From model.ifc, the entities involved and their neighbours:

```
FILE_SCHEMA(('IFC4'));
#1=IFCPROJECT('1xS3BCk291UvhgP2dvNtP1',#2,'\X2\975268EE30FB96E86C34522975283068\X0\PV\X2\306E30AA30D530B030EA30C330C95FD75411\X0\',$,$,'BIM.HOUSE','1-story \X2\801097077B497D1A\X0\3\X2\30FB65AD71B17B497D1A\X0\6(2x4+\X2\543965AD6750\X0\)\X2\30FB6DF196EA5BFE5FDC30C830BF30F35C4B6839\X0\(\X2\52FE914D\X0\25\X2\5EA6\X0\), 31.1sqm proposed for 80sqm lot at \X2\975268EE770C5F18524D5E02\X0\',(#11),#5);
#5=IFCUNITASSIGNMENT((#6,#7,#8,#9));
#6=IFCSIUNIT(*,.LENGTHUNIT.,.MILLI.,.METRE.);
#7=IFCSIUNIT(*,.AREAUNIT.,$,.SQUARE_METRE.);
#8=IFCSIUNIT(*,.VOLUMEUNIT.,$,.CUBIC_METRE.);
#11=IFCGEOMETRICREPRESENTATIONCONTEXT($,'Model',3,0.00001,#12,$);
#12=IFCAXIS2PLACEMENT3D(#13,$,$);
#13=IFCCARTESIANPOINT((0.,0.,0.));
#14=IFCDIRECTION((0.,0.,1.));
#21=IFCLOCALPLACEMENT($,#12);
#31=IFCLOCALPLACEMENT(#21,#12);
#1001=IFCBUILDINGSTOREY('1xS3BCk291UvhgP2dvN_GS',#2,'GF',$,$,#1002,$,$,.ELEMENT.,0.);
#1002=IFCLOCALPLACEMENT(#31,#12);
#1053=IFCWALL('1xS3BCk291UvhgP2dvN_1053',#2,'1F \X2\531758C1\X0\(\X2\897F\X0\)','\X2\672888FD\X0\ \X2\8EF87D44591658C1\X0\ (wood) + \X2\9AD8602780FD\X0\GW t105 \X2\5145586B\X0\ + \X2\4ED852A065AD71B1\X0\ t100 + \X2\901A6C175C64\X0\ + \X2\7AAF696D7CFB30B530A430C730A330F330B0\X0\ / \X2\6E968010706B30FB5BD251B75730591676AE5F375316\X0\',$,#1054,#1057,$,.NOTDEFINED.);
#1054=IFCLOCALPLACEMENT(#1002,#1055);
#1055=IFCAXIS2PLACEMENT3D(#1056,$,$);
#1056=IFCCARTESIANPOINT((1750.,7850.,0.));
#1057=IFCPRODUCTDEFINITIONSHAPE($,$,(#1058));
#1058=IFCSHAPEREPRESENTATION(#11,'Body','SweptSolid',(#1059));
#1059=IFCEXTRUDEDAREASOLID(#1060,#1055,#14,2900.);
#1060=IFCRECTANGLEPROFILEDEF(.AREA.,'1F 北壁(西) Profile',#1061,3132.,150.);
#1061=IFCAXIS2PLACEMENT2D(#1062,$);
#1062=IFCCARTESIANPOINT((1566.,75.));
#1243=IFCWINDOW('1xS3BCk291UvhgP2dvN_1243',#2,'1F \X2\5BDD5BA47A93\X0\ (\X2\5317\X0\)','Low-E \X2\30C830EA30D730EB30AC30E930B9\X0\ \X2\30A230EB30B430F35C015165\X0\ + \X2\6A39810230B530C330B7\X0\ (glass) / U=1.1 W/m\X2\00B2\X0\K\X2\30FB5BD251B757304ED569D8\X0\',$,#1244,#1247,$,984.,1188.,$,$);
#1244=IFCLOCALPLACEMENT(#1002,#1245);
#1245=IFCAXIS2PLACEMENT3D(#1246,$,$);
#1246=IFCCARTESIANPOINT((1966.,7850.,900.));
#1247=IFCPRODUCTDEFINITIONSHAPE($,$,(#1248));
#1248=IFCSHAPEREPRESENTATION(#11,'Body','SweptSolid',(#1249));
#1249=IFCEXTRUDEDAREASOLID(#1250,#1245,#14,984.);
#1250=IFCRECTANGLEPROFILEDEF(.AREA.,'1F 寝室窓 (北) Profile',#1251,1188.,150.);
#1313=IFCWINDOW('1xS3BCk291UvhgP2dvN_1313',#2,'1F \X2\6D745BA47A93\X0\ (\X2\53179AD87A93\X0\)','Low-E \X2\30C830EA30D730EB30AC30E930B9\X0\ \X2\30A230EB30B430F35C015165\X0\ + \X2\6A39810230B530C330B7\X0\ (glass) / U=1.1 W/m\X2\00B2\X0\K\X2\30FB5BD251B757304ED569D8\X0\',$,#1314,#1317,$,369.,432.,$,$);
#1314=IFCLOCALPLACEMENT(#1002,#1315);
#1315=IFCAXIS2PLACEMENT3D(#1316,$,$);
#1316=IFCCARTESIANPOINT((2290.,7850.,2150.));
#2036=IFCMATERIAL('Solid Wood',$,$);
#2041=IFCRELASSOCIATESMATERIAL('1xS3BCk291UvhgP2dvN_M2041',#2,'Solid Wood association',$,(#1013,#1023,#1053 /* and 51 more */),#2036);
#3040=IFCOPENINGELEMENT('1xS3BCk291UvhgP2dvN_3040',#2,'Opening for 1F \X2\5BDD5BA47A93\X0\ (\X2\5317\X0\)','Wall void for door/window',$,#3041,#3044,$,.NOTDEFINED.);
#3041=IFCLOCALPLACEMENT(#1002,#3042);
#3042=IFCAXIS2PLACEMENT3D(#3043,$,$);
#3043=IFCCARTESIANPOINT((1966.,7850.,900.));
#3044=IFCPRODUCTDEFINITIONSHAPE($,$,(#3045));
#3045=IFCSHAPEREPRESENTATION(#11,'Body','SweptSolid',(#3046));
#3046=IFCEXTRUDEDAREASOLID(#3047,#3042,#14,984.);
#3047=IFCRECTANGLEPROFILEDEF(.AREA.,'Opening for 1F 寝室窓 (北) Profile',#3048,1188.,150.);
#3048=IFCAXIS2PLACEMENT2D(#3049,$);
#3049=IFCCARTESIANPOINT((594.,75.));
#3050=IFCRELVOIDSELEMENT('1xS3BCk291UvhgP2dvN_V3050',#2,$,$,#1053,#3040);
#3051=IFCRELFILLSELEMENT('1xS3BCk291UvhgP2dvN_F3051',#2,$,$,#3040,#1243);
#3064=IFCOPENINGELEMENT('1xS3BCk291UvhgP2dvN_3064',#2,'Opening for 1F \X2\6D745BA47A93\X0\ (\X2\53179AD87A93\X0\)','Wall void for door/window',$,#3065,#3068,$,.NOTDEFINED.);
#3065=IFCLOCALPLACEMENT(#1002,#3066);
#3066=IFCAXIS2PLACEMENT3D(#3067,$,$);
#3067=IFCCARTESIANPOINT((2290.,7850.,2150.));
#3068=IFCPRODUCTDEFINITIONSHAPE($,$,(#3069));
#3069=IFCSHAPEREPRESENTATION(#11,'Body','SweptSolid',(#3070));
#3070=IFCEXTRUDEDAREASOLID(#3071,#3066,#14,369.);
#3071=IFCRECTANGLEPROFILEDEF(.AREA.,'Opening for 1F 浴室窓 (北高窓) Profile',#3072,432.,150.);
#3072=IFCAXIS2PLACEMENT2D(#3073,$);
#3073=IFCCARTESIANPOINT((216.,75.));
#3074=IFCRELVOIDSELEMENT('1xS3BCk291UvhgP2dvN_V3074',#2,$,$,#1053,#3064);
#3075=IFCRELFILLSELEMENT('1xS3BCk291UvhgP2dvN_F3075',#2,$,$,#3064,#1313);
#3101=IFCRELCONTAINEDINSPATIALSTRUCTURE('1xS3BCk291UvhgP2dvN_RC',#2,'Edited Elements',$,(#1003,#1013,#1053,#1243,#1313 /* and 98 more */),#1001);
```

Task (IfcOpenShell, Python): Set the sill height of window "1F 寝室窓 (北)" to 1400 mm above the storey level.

```python
import numpy as np
import ifcopenshell
import ifcopenshell.api.geometry
import ifcopenshell.geom
import ifcopenshell.util.element
import ifcopenshell.util.placement
import ifcopenshell.util.shape
import ifcopenshell.util.unit

model = ifcopenshell.open("model.ifc")
unit_scale = ifcopenshell.util.unit.calculate_unit_scale(model)

window = model.by_guid("1xS3BCk291UvhgP2dvN_1243")
opening = window.FillsVoids[0].RelatingOpeningElement
storey = ifcopenshell.util.element.get_container(window, ifc_class="IfcBuildingStorey")
level = ifcopenshell.util.placement.get_local_placement(storey.ObjectPlacement)[2, 3]

# The opening's origin need not be at the sill, so measure its lowest point.
shape = ifcopenshell.geom.create_shape(ifcopenshell.geom.settings(), opening)
bottom = ifcopenshell.util.shape.get_shape_bottom_elevation(shape, shape.geometry) / unit_scale
dz = level + 1.4 / unit_scale - bottom

shift = np.array([0.0, 0.0, dz])
# The window is not placed relative to its opening, so move both.
for product in (opening, window):
    matrix = ifcopenshell.util.placement.get_local_placement(product.ObjectPlacement)
    matrix[:3, 3] += shift
    ifcopenshell.api.geometry.edit_object_placement(model, product=product, matrix=matrix, is_si=False)

print(f"moved by {dz * unit_scale:+.3f} m")

model.write("model_updated.ifc")
```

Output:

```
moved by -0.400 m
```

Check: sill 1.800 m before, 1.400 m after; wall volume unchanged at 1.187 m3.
